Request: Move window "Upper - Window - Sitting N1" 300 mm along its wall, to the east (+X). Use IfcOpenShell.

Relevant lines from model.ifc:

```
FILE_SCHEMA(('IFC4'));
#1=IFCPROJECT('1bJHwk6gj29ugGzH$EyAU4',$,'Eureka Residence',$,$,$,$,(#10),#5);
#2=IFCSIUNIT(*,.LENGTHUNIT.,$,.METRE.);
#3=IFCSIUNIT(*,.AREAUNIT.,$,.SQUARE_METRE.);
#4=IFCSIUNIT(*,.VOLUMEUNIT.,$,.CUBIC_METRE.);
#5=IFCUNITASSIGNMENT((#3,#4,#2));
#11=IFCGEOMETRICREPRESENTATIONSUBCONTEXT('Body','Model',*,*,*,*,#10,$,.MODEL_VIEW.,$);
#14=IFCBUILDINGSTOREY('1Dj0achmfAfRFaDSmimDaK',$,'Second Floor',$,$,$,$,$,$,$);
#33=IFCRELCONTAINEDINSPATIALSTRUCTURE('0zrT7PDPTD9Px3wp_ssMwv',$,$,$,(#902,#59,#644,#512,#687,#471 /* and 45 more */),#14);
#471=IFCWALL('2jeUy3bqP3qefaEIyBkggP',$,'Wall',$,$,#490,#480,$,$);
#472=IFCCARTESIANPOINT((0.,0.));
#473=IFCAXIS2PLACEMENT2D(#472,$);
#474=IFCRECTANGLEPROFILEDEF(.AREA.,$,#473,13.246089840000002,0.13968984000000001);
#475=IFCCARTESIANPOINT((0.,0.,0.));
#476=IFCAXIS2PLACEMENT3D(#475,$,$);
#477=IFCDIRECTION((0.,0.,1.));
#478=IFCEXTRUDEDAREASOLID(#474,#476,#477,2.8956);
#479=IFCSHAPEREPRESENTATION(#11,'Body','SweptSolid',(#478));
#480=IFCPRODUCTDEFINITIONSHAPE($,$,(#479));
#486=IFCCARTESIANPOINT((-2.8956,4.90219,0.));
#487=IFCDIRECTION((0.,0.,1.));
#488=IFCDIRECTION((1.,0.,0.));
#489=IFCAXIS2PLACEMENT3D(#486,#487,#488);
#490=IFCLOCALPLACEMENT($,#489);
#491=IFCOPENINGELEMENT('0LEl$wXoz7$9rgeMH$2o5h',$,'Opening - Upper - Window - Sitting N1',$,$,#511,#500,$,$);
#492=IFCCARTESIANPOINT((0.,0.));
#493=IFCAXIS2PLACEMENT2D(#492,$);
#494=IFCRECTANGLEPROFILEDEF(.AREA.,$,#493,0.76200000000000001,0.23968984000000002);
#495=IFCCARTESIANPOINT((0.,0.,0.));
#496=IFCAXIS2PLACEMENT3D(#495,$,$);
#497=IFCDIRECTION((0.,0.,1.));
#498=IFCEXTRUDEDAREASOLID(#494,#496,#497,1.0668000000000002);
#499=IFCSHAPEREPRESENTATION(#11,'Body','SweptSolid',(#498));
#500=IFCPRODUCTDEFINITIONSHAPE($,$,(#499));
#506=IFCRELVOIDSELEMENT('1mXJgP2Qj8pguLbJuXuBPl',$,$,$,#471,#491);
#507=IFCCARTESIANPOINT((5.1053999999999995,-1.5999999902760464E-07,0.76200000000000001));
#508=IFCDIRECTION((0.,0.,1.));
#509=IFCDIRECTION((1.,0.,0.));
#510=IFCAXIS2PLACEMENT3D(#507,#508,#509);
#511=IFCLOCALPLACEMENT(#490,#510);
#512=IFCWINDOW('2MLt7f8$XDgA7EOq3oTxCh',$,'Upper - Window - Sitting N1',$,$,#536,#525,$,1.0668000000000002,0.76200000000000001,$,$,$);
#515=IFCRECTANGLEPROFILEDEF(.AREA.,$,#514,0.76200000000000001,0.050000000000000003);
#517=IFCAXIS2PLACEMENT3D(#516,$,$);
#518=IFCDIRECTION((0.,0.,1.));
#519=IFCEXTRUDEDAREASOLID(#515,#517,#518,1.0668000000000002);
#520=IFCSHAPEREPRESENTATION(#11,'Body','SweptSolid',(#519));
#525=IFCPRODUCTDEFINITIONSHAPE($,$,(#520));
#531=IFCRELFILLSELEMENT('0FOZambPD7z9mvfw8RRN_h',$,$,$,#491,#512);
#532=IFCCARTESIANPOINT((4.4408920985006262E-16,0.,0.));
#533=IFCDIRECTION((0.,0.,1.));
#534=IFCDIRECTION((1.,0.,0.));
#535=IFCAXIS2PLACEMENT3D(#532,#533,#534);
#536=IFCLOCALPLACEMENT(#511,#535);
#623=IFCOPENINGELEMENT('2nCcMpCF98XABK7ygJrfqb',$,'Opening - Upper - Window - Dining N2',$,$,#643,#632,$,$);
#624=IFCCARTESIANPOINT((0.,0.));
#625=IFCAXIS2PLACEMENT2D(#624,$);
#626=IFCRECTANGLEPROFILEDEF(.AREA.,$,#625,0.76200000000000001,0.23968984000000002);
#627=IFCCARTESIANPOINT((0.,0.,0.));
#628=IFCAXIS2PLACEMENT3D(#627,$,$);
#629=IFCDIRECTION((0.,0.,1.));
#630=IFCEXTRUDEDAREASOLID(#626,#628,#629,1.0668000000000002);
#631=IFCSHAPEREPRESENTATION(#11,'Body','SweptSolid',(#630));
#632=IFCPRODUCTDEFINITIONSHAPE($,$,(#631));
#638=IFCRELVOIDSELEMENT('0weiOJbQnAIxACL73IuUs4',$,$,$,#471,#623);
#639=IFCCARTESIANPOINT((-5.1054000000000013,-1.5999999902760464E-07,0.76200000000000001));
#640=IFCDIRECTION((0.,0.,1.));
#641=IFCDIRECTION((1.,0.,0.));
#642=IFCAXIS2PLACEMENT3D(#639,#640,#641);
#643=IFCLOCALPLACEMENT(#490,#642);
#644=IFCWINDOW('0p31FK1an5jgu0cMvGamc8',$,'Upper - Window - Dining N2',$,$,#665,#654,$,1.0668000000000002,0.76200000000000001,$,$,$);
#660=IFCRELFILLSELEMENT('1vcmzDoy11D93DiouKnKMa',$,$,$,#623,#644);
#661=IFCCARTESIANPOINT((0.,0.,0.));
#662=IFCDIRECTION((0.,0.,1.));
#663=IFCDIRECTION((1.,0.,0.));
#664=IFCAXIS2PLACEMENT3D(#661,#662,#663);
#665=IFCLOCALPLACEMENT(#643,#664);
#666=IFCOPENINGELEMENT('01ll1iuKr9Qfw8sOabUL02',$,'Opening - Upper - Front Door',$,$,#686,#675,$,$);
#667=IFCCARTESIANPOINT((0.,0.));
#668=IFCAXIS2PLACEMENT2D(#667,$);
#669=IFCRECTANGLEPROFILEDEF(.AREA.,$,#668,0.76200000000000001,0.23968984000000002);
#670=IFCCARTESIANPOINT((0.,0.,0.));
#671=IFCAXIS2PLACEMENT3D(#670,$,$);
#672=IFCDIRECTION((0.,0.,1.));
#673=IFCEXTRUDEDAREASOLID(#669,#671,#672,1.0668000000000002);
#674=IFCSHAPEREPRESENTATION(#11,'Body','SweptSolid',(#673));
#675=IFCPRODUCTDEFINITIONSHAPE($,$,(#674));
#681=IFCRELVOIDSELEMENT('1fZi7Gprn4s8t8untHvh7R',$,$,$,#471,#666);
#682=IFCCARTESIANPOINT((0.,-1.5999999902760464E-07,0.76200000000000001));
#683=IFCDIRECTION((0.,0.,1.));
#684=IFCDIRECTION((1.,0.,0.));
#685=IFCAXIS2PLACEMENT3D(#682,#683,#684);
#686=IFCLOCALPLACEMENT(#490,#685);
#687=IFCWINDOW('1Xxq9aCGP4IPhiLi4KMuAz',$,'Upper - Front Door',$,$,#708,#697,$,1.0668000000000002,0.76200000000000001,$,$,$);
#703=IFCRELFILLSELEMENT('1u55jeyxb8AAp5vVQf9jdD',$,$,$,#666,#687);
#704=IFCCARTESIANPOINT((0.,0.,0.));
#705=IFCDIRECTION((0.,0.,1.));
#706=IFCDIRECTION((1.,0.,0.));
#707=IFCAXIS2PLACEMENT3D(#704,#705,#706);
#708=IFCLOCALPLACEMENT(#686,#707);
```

```python
import ifcopenshell
import ifcopenshell.api.geometry
import ifcopenshell.util.placement
import ifcopenshell.util.unit

model = ifcopenshell.open("model.ifc")
unit_scale = ifcopenshell.util.unit.calculate_unit_scale(model)

window = model.by_id(512)
opening = window.FillsVoids[0].RelatingOpeningElement
wall = opening.VoidsElements[0].RelatingBuildingElement

wall_matrix = ifcopenshell.util.placement.get_local_placement(wall.ObjectPlacement)
shift = wall_matrix[:3, 0] * 0.3 / unit_scale
before = ifcopenshell.util.placement.get_local_placement(window.ObjectPlacement)[:3, 3].copy()

# The window is placed relative to its opening, so it follows when the opening moves.
matrix = ifcopenshell.util.placement.get_local_placement(opening.ObjectPlacement)
matrix[:3, 3] += shift
ifcopenshell.api.geometry.edit_object_placement(
    model, product=opening, matrix=matrix, is_si=False, should_transform_children=True
)

after = ifcopenshell.util.placement.get_local_placement(window.ObjectPlacement)[:3, 3]
print("window moved by", (after - before).round(3) + 0.0)

model.write("model_rev.ifc")
```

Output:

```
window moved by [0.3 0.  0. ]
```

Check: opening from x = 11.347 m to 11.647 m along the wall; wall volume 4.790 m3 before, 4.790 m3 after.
